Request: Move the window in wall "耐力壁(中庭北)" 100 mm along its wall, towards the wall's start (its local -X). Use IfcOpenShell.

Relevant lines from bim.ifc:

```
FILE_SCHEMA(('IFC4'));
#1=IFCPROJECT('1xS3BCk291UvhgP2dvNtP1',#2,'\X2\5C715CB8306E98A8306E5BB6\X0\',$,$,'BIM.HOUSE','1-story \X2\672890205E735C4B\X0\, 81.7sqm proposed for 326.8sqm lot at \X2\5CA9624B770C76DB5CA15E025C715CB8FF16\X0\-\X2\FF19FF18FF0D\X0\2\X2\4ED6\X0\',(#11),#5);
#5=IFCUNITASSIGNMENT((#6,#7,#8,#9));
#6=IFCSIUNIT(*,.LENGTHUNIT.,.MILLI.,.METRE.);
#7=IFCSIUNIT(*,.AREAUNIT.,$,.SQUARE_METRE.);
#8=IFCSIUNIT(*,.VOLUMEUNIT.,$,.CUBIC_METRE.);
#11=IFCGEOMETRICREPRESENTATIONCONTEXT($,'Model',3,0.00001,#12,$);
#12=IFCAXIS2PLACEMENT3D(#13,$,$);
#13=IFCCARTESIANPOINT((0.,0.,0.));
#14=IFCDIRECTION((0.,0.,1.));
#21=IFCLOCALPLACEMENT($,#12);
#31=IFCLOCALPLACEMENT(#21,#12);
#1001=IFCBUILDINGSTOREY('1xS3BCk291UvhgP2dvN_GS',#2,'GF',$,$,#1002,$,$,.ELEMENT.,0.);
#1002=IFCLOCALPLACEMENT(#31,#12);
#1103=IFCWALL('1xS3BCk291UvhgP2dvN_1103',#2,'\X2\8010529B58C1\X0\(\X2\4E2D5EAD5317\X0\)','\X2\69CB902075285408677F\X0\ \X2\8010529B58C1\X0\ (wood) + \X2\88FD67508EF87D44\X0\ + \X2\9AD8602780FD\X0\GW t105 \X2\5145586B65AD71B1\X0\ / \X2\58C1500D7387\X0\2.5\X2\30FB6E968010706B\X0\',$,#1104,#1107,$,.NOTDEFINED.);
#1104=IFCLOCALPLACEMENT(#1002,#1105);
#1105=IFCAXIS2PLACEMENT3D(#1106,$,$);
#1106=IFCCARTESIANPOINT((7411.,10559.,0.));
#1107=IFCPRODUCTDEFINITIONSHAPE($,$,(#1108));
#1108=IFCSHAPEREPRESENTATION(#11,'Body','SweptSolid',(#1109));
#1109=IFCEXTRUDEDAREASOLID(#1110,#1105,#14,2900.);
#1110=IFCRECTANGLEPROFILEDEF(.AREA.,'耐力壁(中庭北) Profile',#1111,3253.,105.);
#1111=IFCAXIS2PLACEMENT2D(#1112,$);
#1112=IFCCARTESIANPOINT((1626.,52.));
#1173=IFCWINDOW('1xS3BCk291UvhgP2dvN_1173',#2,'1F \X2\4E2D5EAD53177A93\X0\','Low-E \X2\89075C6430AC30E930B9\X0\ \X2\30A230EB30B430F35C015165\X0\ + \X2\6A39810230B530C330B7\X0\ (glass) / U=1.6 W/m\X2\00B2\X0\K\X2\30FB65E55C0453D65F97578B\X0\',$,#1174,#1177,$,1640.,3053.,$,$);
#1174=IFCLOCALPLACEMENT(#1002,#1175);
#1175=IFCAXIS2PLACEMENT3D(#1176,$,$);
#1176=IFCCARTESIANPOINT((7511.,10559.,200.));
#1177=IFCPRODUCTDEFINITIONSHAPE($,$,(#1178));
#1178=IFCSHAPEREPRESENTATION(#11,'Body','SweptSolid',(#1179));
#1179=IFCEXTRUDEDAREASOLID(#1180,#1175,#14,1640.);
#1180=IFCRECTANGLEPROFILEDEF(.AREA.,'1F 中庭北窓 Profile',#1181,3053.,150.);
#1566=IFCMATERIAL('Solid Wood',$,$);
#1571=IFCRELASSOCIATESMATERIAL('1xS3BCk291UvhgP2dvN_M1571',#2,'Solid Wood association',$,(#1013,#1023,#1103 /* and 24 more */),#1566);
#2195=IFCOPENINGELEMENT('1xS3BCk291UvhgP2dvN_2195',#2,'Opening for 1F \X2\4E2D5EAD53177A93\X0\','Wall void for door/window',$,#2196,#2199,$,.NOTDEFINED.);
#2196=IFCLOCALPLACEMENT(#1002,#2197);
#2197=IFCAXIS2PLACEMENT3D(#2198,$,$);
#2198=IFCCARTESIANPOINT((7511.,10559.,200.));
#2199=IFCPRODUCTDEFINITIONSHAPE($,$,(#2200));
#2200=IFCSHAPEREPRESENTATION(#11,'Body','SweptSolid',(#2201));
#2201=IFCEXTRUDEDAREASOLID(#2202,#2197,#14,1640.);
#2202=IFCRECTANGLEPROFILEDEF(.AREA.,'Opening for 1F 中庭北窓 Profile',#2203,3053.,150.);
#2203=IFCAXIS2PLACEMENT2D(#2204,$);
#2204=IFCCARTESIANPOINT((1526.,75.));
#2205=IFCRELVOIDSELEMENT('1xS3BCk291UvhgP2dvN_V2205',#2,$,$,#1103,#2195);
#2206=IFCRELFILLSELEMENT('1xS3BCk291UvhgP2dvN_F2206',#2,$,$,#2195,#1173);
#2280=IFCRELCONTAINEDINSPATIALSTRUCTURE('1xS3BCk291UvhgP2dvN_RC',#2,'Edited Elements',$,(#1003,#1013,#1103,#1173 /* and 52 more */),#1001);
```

```python
import ifcopenshell
import ifcopenshell.api.geometry
import ifcopenshell.util.placement
import ifcopenshell.util.unit

model = ifcopenshell.open("bim.ifc")
unit_scale = ifcopenshell.util.unit.calculate_unit_scale(model)

window = model.by_guid("1xS3BCk291UvhgP2dvN_1173")
opening = window.FillsVoids[0].RelatingOpeningElement
wall = opening.VoidsElements[0].RelatingBuildingElement

wall_matrix = ifcopenshell.util.placement.get_local_placement(wall.ObjectPlacement)
shift = wall_matrix[:3, 0] * -0.1 / unit_scale
before = ifcopenshell.util.placement.get_local_placement(window.ObjectPlacement)[:3, 3].copy()

# The window is not placed relative to its opening, so move both.
for product in (opening, window):
    matrix = ifcopenshell.util.placement.get_local_placement(product.ObjectPlacement)
    matrix[:3, 3] += shift
    ifcopenshell.api.geometry.edit_object_placement(model, product=product, matrix=matrix, is_si=False)

after = ifcopenshell.util.placement.get_local_placement(window.ObjectPlacement)[:3, 3]
print("window moved by", (after - before).round(3) + 0.0)

model.write("bim_v2.ifc")
```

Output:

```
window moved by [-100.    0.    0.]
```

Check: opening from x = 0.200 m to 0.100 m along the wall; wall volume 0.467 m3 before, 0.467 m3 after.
